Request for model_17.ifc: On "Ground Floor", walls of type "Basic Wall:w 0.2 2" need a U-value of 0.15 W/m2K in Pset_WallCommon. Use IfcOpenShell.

First a look at what the model holds.

```python
import ifcopenshell
import ifcopenshell.util.element

model = ifcopenshell.open("model_17.ifc")
print(model.schema)
storey = next(s for s in model.by_type("IfcBuildingStorey") if s.Name == "Ground Floor")
walls = [e for e in ifcopenshell.util.element.get_decomposition(storey) if e.is_a("IfcWall")]
seen = {}
for e in walls:
    element_type = ifcopenshell.util.element.get_type(e)
    key = (element_type.Name if element_type != e and element_type else None, ifcopenshell.util.element.get_pset(e, "Pset_WallCommon", "ThermalTransmittance"))
    seen[key] = seen.get(key, 0) + 1
for (name, value), count in sorted(seen.items(), key=str):
    print(count, "x", name, "|", value)
```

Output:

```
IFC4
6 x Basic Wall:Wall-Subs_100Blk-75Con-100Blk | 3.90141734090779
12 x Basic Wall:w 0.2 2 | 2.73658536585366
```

```python
import ifcopenshell
import ifcopenshell.api.pset
import ifcopenshell.util.element

model = ifcopenshell.open("model_17.ifc")

storey = next(s for s in model.by_type("IfcBuildingStorey") if s.Name == "Ground Floor")
walls = [e for e in ifcopenshell.util.element.get_decomposition(storey) if e.is_a("IfcWall")]

count = 0
for e in walls:
    element_type = ifcopenshell.util.element.get_type(e)
    if element_type in (None, e) or element_type.Name != "Basic Wall:w 0.2 2":
        continue
    # add_pset returns the element's existing set when there is one.
    pset = ifcopenshell.api.pset.add_pset(model, product=e, name="Pset_WallCommon")
    ifcopenshell.api.pset.edit_pset(model, pset=pset, properties={"ThermalTransmittance": 0.15})
    count += 1

print(count, "walls updated")

model.write("model_17_edited.ifc")
```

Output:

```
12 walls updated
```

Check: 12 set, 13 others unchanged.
